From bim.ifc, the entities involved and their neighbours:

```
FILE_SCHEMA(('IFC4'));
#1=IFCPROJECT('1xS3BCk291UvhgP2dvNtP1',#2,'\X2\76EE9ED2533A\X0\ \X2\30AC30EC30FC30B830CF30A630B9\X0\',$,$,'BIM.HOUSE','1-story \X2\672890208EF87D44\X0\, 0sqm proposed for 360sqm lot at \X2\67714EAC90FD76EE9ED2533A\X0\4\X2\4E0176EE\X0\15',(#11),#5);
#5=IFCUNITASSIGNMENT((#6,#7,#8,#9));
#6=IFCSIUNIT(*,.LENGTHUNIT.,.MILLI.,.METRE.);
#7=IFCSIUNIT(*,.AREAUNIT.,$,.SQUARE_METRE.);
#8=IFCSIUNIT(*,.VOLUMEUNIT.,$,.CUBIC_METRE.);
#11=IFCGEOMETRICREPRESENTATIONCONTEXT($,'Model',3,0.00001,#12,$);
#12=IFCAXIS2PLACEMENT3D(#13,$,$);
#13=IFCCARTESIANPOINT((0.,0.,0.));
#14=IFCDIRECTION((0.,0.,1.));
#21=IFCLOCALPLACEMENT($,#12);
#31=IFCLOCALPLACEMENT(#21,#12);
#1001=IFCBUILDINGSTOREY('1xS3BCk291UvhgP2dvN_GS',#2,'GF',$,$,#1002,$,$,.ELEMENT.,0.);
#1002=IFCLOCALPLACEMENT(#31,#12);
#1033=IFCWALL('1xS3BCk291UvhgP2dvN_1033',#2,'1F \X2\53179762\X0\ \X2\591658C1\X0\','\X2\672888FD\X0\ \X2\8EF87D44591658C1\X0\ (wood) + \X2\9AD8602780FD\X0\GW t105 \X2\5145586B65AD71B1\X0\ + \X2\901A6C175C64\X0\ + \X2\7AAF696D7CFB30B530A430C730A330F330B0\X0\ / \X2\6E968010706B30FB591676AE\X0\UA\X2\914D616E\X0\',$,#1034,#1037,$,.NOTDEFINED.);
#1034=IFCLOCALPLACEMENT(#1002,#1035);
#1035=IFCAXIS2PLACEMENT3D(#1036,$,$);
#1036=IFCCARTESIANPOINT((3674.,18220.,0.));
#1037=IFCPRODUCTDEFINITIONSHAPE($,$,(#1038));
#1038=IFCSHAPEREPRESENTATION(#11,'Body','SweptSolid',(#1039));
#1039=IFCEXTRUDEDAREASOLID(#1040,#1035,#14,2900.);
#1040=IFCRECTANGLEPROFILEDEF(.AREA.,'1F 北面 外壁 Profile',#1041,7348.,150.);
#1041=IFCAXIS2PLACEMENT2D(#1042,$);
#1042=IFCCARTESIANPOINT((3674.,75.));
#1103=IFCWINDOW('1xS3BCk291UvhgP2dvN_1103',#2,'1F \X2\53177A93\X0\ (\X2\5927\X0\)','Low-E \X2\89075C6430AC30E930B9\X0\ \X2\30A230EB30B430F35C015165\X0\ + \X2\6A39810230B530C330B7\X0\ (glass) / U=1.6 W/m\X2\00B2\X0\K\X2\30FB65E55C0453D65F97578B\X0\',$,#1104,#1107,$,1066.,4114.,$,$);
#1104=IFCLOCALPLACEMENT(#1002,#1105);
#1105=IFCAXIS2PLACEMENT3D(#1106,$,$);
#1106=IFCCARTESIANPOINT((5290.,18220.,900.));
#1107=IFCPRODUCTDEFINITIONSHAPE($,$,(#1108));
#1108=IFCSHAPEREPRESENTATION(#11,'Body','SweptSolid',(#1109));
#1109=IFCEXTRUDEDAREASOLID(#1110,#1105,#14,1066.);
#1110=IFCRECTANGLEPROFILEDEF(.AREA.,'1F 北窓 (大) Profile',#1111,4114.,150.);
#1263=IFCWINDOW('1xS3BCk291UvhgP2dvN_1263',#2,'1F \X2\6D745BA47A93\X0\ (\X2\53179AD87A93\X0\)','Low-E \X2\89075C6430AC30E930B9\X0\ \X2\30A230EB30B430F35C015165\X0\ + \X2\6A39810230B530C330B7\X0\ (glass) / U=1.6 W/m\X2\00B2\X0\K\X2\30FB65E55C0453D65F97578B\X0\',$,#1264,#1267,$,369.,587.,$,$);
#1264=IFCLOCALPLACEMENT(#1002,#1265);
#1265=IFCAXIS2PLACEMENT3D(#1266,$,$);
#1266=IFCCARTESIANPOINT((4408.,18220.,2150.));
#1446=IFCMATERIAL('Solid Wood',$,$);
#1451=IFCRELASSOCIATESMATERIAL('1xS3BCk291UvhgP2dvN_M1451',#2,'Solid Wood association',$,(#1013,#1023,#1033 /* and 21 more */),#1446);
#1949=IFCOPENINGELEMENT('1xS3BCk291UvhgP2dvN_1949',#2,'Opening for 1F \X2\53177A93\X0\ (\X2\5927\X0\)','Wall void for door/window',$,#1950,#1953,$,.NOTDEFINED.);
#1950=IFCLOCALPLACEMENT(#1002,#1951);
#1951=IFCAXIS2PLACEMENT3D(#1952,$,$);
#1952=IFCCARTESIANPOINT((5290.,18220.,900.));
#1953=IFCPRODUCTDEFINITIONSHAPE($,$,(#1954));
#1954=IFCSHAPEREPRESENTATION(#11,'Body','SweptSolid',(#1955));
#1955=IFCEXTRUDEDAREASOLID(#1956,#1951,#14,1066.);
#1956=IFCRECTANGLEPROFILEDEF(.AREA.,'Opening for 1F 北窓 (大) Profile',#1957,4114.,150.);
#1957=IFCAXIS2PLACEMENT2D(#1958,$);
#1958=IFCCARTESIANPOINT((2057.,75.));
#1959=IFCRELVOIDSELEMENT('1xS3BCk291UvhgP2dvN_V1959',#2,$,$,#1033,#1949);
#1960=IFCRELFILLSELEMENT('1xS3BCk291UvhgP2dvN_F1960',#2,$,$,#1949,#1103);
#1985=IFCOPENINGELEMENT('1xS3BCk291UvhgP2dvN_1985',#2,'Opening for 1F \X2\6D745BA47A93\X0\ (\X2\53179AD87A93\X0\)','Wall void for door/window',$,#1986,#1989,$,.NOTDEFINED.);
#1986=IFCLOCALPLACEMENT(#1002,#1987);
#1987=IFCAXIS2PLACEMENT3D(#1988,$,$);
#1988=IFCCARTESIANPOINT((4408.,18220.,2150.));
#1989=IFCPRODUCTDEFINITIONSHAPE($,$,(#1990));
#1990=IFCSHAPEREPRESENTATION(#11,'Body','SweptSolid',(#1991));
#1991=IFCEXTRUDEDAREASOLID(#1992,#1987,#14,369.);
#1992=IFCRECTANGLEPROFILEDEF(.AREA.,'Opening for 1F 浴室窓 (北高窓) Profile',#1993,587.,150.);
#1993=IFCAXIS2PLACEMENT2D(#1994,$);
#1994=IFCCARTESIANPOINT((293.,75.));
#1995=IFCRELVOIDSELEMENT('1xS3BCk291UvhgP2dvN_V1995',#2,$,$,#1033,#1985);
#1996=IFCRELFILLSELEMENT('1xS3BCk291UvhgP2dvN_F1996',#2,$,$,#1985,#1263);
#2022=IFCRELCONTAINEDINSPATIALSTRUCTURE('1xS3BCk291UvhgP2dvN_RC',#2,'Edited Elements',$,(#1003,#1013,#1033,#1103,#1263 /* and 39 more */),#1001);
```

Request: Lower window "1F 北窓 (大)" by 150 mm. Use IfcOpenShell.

```python
import numpy as np
import ifcopenshell
import ifcopenshell.api.geometry
import ifcopenshell.util.placement
import ifcopenshell.util.unit

model = ifcopenshell.open("bim.ifc")
unit_scale = ifcopenshell.util.unit.calculate_unit_scale(model)

window = model.by_guid("1xS3BCk291UvhgP2dvN_1103")
opening = window.FillsVoids[0].RelatingOpeningElement
dz = -0.15 / unit_scale

shift = np.array([0.0, 0.0, dz])
# The window is not placed relative to its opening, so move both.
for product in (opening, window):
    matrix = ifcopenshell.util.placement.get_local_placement(product.ObjectPlacement)
    matrix[:3, 3] += shift
    ifcopenshell.api.geometry.edit_object_placement(model, product=product, matrix=matrix, is_si=False)

print(f"moved by {dz * unit_scale:+.3f} m")

model.write("bim_v2.ifc")
```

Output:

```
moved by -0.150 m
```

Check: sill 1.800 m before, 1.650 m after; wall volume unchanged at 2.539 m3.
